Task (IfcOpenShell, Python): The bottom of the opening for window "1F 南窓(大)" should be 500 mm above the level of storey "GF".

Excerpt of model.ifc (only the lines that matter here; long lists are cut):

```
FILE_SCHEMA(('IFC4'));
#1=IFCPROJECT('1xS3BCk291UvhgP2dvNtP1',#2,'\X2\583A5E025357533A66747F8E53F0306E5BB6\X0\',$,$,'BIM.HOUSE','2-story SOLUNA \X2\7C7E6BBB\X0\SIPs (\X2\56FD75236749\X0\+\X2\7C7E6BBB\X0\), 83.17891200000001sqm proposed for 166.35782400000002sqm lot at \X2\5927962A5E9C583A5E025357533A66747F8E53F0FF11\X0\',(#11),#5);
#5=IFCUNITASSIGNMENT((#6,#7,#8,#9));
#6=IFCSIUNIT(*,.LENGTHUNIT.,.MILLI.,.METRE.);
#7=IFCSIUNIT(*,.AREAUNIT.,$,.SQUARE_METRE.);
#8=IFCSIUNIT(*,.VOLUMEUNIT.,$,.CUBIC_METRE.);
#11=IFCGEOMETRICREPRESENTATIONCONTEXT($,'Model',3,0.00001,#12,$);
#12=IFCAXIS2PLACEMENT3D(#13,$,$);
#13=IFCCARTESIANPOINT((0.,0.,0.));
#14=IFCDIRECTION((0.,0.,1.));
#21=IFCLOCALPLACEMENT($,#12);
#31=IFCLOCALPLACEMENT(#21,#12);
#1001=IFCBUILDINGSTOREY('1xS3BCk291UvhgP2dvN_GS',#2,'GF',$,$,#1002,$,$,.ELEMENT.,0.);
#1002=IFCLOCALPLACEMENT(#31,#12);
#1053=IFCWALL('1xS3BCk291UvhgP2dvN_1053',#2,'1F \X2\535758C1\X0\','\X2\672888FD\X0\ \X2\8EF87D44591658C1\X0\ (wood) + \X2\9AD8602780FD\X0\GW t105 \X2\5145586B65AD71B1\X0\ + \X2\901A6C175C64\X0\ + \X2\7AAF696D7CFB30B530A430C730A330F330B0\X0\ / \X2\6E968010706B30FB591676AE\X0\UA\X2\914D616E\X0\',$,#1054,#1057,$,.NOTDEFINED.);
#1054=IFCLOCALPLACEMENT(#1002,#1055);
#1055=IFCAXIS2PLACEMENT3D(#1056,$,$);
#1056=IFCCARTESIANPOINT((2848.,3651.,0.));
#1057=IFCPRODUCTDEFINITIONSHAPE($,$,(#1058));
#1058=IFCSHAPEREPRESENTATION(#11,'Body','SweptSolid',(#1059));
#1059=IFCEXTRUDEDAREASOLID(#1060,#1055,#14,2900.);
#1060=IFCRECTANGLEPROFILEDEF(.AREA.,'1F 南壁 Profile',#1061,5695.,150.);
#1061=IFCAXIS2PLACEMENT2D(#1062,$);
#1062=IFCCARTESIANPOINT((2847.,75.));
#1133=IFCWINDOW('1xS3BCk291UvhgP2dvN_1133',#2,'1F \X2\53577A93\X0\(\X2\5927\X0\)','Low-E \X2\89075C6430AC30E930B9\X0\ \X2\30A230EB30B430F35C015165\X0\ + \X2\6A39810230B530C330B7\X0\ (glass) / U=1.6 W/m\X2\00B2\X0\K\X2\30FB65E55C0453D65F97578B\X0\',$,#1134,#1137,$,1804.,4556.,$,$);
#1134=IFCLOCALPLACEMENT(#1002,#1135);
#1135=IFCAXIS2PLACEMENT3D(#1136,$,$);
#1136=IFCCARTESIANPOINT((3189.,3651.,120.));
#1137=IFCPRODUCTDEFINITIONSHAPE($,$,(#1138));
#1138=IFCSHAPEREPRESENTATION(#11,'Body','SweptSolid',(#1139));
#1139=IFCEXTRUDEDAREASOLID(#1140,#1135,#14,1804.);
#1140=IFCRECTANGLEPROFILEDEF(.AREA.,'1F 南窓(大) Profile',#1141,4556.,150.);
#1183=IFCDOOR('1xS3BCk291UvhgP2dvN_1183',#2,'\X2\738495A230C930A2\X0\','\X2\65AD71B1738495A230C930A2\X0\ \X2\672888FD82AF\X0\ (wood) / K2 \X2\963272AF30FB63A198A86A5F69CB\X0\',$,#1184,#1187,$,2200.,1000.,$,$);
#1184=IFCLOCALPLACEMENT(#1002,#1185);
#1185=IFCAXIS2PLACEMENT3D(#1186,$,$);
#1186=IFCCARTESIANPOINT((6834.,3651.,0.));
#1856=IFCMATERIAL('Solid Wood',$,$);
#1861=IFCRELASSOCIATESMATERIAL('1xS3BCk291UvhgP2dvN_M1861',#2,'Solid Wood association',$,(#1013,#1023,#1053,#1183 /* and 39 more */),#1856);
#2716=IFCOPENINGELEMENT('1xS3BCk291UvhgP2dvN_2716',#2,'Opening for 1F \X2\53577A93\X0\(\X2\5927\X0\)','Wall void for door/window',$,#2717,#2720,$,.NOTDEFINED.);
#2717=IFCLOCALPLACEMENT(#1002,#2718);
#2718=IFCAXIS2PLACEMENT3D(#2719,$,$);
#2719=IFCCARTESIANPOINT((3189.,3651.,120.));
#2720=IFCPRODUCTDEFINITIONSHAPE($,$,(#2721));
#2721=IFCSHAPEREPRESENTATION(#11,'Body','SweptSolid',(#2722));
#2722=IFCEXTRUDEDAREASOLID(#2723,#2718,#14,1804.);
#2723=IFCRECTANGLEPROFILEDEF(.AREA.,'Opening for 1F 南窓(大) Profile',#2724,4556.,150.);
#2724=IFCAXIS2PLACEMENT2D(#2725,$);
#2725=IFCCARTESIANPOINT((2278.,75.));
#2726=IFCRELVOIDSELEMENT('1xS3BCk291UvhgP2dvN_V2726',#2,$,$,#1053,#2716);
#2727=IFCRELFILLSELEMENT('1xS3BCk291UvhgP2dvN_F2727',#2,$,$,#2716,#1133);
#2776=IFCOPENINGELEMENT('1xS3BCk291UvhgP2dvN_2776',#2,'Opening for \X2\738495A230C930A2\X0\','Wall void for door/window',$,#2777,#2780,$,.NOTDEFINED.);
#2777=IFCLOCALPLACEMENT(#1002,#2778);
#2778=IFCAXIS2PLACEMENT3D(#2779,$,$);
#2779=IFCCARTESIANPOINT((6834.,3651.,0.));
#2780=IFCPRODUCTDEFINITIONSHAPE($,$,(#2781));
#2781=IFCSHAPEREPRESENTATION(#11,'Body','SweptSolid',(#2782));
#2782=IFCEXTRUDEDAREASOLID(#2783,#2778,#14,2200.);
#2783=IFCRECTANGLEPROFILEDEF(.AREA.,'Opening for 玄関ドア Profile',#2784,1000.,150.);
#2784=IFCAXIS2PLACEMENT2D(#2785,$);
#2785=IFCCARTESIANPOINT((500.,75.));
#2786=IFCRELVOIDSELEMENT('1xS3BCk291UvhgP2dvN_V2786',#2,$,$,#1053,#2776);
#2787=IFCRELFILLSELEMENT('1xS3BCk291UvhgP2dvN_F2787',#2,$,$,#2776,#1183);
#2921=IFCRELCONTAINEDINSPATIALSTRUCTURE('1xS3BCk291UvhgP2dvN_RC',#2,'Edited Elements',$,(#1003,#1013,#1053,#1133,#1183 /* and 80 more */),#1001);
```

```python
import numpy as np
import ifcopenshell
import ifcopenshell.api.geometry
import ifcopenshell.geom
import ifcopenshell.util.element
import ifcopenshell.util.placement
import ifcopenshell.util.shape
import ifcopenshell.util.unit

model = ifcopenshell.open("model.ifc")
unit_scale = ifcopenshell.util.unit.calculate_unit_scale(model)

window = model.by_guid("1xS3BCk291UvhgP2dvN_1133")
opening = window.FillsVoids[0].RelatingOpeningElement
storey = ifcopenshell.util.element.get_container(window, ifc_class="IfcBuildingStorey")
level = ifcopenshell.util.placement.get_local_placement(storey.ObjectPlacement)[2, 3]

# The opening's origin need not be at the sill, so measure its lowest point.
shape = ifcopenshell.geom.create_shape(ifcopenshell.geom.settings(), opening)
bottom = ifcopenshell.util.shape.get_shape_bottom_elevation(shape, shape.geometry) / unit_scale
dz = level + 0.5 / unit_scale - bottom

shift = np.array([0.0, 0.0, dz])
# The window is not placed relative to its opening, so move both.
for product in (opening, window):
    matrix = ifcopenshell.util.placement.get_local_placement(product.ObjectPlacement)
    matrix[:3, 3] += shift
    ifcopenshell.api.geometry.edit_object_placement(model, product=product, matrix=matrix, is_si=False)

print(f"moved by {dz * unit_scale:+.3f} m")

model.write("model_rev.ifc")
```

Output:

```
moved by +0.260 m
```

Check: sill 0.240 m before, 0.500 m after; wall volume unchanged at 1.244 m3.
